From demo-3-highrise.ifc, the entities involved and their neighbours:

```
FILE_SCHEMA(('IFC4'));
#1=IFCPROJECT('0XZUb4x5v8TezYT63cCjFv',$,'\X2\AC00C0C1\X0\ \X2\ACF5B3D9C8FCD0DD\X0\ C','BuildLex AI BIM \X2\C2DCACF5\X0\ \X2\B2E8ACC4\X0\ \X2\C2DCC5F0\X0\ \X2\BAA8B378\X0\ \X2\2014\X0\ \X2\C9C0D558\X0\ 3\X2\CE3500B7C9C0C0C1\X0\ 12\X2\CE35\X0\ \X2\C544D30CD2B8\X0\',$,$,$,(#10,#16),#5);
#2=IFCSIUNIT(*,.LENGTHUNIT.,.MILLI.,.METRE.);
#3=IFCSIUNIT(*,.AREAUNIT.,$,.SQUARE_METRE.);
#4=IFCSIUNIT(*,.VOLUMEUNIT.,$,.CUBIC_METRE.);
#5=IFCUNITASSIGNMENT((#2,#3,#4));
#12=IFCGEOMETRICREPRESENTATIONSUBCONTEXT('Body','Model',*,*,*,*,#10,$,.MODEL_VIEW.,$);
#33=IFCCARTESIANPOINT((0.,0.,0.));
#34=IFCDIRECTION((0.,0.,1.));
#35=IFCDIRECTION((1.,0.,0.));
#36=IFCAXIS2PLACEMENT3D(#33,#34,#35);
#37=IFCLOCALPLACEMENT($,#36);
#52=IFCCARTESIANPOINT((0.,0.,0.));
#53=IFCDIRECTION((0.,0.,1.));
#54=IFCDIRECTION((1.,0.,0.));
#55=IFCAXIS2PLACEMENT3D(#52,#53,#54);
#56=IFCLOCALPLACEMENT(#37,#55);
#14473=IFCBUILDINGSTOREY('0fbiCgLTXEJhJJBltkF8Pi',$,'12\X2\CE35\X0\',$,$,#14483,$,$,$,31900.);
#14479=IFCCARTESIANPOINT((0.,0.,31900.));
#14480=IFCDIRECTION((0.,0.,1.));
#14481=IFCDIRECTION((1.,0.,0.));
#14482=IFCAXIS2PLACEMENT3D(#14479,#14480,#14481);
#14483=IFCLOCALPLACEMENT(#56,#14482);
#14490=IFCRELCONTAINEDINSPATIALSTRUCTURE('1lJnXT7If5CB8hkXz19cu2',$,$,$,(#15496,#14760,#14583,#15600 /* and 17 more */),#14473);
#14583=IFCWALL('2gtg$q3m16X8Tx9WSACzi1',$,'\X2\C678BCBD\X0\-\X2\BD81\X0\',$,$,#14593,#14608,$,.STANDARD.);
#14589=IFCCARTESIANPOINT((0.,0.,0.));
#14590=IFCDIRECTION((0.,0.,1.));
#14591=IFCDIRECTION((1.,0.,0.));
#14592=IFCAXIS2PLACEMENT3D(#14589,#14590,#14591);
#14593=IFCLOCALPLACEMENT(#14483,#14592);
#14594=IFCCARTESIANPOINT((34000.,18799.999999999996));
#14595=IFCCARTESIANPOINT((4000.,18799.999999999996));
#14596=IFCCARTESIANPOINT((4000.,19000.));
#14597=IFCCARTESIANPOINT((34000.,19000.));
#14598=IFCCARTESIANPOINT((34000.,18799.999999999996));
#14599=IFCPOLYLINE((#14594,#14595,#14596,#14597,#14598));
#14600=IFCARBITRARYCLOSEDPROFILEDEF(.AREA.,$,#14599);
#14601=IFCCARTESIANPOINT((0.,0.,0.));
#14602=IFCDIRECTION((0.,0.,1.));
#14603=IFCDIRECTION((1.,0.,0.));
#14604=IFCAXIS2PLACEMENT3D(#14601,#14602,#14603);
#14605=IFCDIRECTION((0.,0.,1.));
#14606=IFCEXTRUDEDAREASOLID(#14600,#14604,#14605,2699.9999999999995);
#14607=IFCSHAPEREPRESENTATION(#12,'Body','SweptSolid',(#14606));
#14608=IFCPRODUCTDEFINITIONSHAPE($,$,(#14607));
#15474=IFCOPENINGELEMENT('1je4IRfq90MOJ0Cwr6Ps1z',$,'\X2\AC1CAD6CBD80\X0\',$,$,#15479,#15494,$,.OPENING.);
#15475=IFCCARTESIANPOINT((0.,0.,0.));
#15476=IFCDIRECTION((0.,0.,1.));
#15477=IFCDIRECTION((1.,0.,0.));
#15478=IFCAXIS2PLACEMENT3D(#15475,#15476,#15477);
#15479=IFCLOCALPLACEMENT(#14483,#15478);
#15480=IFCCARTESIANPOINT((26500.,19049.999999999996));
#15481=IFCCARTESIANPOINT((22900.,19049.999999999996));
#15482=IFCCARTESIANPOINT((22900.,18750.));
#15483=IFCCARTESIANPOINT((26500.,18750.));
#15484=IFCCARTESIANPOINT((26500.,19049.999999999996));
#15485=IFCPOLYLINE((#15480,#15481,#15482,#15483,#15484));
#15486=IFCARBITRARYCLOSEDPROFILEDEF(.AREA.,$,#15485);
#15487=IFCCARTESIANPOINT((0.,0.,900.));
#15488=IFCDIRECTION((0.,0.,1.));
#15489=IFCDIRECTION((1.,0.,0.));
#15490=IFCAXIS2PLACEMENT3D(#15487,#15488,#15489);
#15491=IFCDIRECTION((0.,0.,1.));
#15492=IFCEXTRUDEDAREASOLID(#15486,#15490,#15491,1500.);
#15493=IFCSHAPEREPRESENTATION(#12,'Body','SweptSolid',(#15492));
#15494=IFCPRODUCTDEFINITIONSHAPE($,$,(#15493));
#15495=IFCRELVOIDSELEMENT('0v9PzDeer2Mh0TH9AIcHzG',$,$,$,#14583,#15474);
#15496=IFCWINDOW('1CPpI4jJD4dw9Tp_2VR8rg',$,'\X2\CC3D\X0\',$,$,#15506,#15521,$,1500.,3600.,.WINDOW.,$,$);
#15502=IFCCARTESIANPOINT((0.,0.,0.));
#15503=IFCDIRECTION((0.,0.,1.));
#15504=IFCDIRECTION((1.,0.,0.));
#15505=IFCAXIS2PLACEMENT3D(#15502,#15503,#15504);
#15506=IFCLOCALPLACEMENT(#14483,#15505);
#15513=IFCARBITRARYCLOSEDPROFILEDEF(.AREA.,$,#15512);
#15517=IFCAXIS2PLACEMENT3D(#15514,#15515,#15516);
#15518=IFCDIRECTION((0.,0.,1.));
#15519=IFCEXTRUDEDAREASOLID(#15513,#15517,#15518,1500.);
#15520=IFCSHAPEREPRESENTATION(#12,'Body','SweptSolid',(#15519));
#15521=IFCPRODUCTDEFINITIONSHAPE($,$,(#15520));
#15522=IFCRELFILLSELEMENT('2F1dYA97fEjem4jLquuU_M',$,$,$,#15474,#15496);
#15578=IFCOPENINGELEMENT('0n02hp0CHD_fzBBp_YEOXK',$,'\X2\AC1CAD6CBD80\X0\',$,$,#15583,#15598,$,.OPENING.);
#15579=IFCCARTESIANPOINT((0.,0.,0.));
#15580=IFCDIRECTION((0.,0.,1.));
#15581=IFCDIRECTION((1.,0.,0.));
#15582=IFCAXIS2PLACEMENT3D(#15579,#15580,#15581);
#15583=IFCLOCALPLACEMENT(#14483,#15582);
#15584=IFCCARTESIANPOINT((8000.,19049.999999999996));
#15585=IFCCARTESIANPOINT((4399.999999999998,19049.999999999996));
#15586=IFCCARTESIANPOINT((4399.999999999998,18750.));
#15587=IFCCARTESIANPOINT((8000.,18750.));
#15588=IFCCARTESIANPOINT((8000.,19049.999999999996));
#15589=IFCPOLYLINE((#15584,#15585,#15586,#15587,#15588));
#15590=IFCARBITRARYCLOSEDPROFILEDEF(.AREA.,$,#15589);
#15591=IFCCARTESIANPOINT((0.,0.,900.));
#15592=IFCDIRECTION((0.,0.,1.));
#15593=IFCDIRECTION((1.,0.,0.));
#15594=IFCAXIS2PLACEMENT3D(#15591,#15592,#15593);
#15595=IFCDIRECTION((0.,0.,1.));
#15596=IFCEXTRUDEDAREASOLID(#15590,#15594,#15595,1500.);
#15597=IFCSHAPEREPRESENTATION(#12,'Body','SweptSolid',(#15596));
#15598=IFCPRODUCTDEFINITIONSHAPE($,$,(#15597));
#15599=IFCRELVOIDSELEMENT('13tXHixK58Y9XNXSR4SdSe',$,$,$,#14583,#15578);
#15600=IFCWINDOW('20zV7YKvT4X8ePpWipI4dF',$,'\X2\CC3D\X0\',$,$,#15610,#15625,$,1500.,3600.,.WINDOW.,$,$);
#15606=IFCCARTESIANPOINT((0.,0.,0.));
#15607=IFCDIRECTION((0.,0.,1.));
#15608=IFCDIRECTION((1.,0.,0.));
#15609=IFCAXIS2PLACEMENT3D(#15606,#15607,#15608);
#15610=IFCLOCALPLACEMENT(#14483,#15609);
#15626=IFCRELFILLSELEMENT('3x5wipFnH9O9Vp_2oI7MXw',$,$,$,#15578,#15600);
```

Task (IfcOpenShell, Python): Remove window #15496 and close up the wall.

```python
import ifcopenshell
import ifcopenshell.api.feature
import ifcopenshell.api.root
import ifcopenshell.geom
import ifcopenshell.util.shape

model = ifcopenshell.open("demo-3-highrise.ifc")
settings = ifcopenshell.geom.settings()


def volume(element):
    """Net volume in cubic metres, openings subtracted."""
    shape = ifcopenshell.geom.create_shape(settings, element)
    return ifcopenshell.util.shape.get_volume(shape.geometry)


window = model.by_guid("1CPpI4jJD4dw9Tp_2VR8rg")
opening = window.FillsVoids[0].RelatingOpeningElement
wall = opening.VoidsElements[0].RelatingBuildingElement
before = volume(wall)

ifcopenshell.api.root.remove_product(model, product=window)
ifcopenshell.api.feature.remove_feature(model, feature=opening)

after = volume(wall)

print(f"wall volume {before:.3f} -> {after:.3f} m3")

model.write("demo-3-highrise_v2.ifc")
```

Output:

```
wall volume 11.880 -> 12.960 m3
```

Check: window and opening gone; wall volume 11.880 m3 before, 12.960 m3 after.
